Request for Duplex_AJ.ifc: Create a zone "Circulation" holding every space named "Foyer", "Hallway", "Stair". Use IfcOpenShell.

First a look at what the model holds.

```python
import ifcopenshell

model = ifcopenshell.open("Duplex_AJ.ifc")
print(model.schema)
seen = {}
for space in model.by_type("IfcSpace"):
    seen[space.LongName] = seen.get(space.LongName, 0) + 1
for name, count in sorted(seen.items(), key=str):
    print(count, "x", name)
print("zones:", [z.Name for z in model.by_type("IfcZone")][:20])
```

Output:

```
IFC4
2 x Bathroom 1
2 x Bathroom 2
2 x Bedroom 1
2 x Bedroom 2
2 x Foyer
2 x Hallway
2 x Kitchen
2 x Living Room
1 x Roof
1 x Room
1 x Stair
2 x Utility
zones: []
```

```python
import ifcopenshell
import ifcopenshell.api.group
import ifcopenshell.api.root

model = ifcopenshell.open("Duplex_AJ.ifc")

names = {"Foyer", "Hallway", "Stair"}
spaces = [s for s in model.by_type("IfcSpace") if s.LongName in names]

zone = ifcopenshell.api.root.create_entity(model, ifc_class="IfcZone", name="Circulation")
ifcopenshell.api.group.assign_group(model, products=spaces, group=zone)
print(len(spaces), "spaces in", zone.Name)

model.write("Duplex_AJ_updated.ifc")
```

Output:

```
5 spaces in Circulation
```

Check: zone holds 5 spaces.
